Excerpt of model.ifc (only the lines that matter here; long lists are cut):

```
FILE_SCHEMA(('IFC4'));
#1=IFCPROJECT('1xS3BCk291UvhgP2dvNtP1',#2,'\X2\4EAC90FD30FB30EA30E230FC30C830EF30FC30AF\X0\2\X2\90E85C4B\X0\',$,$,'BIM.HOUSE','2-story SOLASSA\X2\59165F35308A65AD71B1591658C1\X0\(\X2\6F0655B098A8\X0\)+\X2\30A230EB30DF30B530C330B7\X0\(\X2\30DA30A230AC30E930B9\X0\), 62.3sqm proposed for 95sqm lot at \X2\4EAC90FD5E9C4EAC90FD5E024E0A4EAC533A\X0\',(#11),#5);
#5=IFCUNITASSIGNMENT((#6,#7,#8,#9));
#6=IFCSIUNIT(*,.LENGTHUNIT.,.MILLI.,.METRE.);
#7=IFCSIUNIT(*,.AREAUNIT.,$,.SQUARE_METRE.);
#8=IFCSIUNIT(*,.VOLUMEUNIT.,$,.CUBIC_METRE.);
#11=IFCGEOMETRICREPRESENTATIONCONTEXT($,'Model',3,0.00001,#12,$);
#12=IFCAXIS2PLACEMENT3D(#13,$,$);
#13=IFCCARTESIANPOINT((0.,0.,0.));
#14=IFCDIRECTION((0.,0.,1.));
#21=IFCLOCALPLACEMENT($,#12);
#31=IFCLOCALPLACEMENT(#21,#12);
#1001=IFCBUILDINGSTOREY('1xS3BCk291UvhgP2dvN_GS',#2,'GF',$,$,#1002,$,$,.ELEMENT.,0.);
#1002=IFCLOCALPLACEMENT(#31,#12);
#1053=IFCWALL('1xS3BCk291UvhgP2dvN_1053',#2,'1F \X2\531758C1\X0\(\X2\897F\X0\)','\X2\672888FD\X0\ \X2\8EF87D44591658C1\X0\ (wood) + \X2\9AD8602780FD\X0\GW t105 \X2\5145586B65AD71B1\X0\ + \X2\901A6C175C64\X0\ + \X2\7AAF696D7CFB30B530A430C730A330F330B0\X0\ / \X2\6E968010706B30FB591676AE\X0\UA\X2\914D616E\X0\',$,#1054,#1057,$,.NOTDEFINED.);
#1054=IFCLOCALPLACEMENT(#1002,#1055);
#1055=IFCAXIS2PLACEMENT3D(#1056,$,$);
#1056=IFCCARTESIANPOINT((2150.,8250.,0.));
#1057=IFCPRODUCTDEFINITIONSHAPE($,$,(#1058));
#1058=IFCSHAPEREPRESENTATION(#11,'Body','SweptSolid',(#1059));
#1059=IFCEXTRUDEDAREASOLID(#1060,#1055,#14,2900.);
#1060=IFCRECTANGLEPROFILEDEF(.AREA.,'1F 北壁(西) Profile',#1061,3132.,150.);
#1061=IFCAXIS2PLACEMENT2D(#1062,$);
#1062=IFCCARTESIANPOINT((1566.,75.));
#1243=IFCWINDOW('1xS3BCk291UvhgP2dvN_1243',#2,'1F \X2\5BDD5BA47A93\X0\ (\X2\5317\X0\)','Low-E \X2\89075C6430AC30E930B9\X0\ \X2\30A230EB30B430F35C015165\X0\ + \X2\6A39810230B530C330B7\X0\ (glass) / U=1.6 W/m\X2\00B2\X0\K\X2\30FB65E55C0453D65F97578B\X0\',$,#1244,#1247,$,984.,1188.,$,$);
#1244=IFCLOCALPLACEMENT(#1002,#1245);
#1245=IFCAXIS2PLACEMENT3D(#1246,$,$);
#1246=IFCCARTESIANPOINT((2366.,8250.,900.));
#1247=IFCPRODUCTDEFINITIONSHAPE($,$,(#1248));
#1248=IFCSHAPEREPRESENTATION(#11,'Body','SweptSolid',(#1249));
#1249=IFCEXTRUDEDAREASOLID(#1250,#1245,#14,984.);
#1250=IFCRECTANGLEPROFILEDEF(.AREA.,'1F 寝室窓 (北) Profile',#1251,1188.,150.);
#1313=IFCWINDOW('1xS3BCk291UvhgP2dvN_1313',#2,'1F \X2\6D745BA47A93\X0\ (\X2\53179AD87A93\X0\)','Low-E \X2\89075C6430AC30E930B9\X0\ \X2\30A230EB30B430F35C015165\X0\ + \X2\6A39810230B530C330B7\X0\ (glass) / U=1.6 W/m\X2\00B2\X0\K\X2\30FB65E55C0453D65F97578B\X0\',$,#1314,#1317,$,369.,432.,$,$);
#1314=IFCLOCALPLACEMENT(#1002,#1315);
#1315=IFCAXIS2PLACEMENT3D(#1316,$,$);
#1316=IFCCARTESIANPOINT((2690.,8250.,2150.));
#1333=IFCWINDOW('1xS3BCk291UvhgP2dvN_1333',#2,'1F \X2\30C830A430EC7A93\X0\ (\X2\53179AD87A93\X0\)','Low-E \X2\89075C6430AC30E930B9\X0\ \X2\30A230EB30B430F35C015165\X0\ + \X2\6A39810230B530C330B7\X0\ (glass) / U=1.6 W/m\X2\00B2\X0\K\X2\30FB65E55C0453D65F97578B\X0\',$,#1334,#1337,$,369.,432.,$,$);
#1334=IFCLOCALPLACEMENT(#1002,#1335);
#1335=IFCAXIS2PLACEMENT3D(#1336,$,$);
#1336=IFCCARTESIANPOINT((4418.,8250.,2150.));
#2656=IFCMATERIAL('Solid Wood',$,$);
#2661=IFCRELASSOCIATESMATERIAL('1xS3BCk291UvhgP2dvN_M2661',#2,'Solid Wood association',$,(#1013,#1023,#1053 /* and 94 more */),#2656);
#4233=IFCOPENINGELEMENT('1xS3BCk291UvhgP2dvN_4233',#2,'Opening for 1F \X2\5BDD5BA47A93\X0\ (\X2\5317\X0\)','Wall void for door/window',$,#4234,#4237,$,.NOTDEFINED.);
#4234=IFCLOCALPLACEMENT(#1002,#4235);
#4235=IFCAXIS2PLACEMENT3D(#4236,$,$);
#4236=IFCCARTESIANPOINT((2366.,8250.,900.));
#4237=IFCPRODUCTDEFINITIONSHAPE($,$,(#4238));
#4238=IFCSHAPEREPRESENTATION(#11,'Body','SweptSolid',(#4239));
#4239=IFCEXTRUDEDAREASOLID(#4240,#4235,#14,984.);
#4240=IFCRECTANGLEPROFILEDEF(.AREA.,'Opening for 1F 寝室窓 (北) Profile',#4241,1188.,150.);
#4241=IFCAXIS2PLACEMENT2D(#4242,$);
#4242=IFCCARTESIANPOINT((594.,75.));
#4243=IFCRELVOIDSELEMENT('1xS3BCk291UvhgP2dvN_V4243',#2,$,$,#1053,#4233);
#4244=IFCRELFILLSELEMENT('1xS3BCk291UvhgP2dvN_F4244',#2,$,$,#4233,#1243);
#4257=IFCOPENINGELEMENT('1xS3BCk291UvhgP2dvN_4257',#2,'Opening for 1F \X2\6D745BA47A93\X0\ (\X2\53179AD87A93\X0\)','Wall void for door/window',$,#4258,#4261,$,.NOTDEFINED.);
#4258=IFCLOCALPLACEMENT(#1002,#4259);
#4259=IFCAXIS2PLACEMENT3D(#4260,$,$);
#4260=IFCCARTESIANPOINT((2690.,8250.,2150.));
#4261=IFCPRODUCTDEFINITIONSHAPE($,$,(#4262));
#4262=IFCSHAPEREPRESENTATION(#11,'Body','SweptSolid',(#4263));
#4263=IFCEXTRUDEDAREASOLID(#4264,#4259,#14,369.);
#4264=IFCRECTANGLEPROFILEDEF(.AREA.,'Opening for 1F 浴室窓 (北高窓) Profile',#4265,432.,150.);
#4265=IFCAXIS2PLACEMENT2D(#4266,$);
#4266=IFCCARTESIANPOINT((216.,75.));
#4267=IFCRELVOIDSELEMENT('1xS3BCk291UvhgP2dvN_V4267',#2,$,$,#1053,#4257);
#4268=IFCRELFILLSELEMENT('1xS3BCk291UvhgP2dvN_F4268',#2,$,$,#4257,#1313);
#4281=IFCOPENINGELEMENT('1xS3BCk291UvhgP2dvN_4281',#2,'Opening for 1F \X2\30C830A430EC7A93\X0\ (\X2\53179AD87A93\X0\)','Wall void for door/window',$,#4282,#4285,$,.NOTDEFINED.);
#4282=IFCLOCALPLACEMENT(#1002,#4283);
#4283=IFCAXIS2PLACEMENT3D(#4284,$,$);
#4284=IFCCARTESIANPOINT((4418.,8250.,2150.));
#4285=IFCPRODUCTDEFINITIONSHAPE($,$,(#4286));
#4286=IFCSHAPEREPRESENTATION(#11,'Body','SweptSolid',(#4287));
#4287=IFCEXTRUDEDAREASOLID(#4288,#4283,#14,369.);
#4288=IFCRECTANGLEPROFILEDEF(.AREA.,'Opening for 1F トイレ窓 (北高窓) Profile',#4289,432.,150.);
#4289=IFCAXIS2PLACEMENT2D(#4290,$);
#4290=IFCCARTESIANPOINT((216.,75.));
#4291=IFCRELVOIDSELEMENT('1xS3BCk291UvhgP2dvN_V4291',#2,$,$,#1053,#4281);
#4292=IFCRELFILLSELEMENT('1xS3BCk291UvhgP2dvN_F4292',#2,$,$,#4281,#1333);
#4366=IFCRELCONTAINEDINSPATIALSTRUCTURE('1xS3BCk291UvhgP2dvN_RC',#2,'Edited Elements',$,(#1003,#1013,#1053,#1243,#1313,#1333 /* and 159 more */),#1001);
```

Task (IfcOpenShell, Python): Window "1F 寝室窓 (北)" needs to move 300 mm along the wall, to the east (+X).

```python
import ifcopenshell
import ifcopenshell.api.geometry
import ifcopenshell.util.placement

model = ifcopenshell.open("model.ifc")

window = model.by_guid("1xS3BCk291UvhgP2dvN_1243")
opening = window.FillsVoids[0].RelatingOpeningElement
wall = opening.VoidsElements[0].RelatingBuildingElement

wall_matrix = ifcopenshell.util.placement.get_local_placement(wall.ObjectPlacement)
shift = wall_matrix[:3, 0] * 300.0
before = ifcopenshell.util.placement.get_local_placement(window.ObjectPlacement)[:3, 3].copy()

# The window is not placed relative to its opening, so move both.
for product in (opening, window):
    matrix = ifcopenshell.util.placement.get_local_placement(product.ObjectPlacement)
    matrix[:3, 3] += shift
    ifcopenshell.api.geometry.edit_object_placement(model, product=product, matrix=matrix, is_si=False)

after = ifcopenshell.util.placement.get_local_placement(window.ObjectPlacement)[:3, 3]
print("window moved by", (after - before).round(3) + 0.0)

model.write("model_edited.ifc")
```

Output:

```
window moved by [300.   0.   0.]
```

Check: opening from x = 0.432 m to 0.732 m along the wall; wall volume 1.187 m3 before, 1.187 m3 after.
